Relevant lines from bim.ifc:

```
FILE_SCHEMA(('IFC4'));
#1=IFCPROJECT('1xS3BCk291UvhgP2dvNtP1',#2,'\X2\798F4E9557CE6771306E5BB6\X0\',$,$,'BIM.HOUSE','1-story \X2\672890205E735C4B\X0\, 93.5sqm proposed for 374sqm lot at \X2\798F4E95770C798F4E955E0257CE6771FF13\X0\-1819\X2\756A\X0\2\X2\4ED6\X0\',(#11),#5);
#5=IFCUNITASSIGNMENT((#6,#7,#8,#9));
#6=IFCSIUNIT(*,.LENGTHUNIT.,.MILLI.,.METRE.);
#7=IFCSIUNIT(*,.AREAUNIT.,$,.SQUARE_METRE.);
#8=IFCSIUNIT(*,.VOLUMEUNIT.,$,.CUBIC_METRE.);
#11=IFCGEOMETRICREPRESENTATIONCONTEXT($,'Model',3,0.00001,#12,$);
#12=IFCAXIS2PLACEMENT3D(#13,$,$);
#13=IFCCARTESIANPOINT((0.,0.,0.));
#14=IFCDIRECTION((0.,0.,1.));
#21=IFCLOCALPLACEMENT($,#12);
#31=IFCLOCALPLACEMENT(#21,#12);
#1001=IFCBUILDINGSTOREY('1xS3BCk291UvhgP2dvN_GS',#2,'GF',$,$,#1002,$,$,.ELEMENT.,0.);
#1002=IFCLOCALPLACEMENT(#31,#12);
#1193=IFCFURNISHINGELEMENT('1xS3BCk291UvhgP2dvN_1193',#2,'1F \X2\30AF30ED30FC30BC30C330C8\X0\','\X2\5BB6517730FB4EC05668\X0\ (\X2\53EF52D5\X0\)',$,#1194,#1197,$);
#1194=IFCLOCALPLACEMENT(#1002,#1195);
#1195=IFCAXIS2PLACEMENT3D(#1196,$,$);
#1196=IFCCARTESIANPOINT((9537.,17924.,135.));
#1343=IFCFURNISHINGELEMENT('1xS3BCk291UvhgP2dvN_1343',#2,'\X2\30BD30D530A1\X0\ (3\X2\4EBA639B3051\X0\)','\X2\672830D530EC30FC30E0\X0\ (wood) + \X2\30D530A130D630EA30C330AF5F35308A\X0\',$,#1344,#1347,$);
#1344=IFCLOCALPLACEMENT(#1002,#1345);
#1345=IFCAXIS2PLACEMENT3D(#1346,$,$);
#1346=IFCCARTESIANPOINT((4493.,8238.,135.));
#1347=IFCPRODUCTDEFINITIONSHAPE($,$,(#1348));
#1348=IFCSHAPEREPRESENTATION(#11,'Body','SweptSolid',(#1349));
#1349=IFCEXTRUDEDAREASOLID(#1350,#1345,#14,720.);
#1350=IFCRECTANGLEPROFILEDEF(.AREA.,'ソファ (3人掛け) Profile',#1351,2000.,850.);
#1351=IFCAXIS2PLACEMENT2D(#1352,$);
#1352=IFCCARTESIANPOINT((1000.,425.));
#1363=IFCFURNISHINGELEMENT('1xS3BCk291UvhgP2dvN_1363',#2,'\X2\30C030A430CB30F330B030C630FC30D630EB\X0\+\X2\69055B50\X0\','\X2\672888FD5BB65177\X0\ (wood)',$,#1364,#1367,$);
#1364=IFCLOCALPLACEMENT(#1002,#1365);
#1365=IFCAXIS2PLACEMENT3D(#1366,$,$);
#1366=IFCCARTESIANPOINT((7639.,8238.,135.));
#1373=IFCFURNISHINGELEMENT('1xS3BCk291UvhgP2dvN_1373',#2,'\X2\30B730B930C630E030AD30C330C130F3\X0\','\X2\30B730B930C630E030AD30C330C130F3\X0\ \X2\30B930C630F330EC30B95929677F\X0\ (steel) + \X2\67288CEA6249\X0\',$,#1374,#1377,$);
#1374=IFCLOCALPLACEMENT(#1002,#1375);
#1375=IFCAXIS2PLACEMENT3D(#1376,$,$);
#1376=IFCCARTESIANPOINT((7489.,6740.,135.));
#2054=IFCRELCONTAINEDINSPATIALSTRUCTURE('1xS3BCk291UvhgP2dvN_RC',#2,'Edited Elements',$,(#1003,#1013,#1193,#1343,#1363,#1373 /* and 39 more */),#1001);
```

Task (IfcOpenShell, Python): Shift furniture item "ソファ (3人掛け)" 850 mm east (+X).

```python
import ifcopenshell
import ifcopenshell.api.geometry
import ifcopenshell.util.placement

model = ifcopenshell.open("bim.ifc")

item = model.by_guid("1xS3BCk291UvhgP2dvN_1343")
matrix = ifcopenshell.util.placement.get_local_placement(item.ObjectPlacement)
matrix[0, 3] += 850.0
ifcopenshell.api.geometry.edit_object_placement(model, product=item, matrix=matrix, is_si=False)

print(ifcopenshell.util.placement.get_local_placement(item.ObjectPlacement).round(3) + 0.0)

model.write("bim-out.ifc")
```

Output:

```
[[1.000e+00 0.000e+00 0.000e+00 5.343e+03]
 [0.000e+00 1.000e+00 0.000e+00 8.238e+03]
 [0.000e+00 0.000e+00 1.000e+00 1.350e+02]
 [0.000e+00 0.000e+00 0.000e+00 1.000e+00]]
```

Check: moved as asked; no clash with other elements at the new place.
